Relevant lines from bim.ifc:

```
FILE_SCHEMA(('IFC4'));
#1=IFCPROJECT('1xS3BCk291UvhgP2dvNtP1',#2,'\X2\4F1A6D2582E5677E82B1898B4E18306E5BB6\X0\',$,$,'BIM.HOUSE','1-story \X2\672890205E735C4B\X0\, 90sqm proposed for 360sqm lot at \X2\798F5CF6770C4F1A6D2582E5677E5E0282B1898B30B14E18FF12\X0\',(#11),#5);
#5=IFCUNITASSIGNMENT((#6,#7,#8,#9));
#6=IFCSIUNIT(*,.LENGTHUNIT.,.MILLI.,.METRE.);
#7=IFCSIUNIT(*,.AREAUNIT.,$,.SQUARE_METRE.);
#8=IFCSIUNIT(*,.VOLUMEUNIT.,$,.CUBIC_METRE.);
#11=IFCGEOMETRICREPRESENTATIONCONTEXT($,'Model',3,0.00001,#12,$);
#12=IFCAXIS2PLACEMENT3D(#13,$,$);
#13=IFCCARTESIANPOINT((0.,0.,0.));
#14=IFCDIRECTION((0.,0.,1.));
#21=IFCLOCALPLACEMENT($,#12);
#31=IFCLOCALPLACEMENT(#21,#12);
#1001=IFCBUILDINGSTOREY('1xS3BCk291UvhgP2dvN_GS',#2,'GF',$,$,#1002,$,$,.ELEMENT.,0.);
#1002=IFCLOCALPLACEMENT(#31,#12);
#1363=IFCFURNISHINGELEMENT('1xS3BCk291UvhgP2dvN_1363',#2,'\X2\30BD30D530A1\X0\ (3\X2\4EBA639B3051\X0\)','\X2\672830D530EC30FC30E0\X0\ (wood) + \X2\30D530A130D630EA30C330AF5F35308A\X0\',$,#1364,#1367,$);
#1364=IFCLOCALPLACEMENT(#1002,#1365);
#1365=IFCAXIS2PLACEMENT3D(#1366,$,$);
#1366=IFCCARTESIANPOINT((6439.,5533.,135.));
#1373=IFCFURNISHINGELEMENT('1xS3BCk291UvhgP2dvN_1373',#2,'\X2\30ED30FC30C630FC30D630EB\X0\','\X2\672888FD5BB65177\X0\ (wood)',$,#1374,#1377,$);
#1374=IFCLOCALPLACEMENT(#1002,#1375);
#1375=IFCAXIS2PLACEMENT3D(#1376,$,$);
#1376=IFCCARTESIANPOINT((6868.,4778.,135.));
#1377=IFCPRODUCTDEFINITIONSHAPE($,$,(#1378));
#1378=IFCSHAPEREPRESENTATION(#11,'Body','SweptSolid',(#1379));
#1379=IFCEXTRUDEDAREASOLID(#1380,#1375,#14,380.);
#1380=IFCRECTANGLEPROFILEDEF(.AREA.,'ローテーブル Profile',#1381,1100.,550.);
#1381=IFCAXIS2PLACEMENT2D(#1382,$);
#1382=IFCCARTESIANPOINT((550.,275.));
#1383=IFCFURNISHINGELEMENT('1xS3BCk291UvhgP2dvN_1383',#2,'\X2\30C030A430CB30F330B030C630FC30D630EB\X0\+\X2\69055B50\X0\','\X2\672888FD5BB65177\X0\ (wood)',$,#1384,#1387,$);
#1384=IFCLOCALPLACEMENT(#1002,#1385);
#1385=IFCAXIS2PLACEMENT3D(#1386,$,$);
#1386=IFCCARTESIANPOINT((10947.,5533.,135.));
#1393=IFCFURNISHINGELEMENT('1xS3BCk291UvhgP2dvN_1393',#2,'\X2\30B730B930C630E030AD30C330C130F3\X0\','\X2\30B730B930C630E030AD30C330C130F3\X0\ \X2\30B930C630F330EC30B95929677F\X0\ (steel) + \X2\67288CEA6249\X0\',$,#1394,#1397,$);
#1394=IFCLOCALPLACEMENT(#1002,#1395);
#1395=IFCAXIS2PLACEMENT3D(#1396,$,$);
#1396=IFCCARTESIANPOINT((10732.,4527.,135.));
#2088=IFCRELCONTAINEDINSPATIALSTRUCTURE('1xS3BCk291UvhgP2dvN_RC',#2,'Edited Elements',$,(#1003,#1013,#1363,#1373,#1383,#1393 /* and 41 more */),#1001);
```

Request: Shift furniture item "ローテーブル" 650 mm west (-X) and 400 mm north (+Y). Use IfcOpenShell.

```python
import ifcopenshell
import ifcopenshell.api.geometry
import ifcopenshell.util.placement
import ifcopenshell.util.unit

model = ifcopenshell.open("bim.ifc")
unit_scale = ifcopenshell.util.unit.calculate_unit_scale(model)

item = model.by_guid("1xS3BCk291UvhgP2dvN_1373")
matrix = ifcopenshell.util.placement.get_local_placement(item.ObjectPlacement)
matrix[0, 3] -= 0.65 / unit_scale
matrix[1, 3] += 0.4 / unit_scale
ifcopenshell.api.geometry.edit_object_placement(model, product=item, matrix=matrix, is_si=False)

print(ifcopenshell.util.placement.get_local_placement(item.ObjectPlacement).round(3) + 0.0)

model.write("bim_rev.ifc")
```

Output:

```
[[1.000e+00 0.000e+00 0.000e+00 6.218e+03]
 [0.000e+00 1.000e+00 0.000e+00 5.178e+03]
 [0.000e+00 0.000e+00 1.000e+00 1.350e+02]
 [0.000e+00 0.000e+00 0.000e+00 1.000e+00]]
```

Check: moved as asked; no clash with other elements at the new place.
